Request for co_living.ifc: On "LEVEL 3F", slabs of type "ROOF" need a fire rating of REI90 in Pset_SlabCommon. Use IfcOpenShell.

First a look at what the model holds.

```python
import ifcopenshell
import ifcopenshell.util.element

model = ifcopenshell.open("co_living.ifc")
print(model.schema)
storey = next(s for s in model.by_type("IfcBuildingStorey") if s.Name == "LEVEL 3F")
slabs = [e for e in ifcopenshell.util.element.get_decomposition(storey) if e.is_a("IfcSlab")]
seen = {}
for e in slabs:
    element_type = ifcopenshell.util.element.get_type(e)
    key = (element_type.Name if element_type != e and element_type else None, ifcopenshell.util.element.get_pset(e, "Pset_SlabCommon", "FireRating"))
    seen[key] = seen.get(key, 0) + 1
for (name, value), count in sorted(seen.items(), key=str):
    print(count, "x", name, "|", value)
```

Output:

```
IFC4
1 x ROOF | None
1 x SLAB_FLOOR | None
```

```python
import ifcopenshell
import ifcopenshell.api.pset
import ifcopenshell.util.element

model = ifcopenshell.open("co_living.ifc")

storey = next(s for s in model.by_type("IfcBuildingStorey") if s.Name == "LEVEL 3F")
slabs = [e for e in ifcopenshell.util.element.get_decomposition(storey) if e.is_a("IfcSlab")]

count = 0
for e in slabs:
    element_type = ifcopenshell.util.element.get_type(e)
    if element_type in (None, e) or element_type.Name != "ROOF":
        continue
    # add_pset returns the element's existing set when there is one.
    pset = ifcopenshell.api.pset.add_pset(model, product=e, name="Pset_SlabCommon")
    ifcopenshell.api.pset.edit_pset(model, pset=pset, properties={"FireRating": "REI90"})
    count += 1

print(count, "slabs updated")

model.write("co_living_v2.ifc")
```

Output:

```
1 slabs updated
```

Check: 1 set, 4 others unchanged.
